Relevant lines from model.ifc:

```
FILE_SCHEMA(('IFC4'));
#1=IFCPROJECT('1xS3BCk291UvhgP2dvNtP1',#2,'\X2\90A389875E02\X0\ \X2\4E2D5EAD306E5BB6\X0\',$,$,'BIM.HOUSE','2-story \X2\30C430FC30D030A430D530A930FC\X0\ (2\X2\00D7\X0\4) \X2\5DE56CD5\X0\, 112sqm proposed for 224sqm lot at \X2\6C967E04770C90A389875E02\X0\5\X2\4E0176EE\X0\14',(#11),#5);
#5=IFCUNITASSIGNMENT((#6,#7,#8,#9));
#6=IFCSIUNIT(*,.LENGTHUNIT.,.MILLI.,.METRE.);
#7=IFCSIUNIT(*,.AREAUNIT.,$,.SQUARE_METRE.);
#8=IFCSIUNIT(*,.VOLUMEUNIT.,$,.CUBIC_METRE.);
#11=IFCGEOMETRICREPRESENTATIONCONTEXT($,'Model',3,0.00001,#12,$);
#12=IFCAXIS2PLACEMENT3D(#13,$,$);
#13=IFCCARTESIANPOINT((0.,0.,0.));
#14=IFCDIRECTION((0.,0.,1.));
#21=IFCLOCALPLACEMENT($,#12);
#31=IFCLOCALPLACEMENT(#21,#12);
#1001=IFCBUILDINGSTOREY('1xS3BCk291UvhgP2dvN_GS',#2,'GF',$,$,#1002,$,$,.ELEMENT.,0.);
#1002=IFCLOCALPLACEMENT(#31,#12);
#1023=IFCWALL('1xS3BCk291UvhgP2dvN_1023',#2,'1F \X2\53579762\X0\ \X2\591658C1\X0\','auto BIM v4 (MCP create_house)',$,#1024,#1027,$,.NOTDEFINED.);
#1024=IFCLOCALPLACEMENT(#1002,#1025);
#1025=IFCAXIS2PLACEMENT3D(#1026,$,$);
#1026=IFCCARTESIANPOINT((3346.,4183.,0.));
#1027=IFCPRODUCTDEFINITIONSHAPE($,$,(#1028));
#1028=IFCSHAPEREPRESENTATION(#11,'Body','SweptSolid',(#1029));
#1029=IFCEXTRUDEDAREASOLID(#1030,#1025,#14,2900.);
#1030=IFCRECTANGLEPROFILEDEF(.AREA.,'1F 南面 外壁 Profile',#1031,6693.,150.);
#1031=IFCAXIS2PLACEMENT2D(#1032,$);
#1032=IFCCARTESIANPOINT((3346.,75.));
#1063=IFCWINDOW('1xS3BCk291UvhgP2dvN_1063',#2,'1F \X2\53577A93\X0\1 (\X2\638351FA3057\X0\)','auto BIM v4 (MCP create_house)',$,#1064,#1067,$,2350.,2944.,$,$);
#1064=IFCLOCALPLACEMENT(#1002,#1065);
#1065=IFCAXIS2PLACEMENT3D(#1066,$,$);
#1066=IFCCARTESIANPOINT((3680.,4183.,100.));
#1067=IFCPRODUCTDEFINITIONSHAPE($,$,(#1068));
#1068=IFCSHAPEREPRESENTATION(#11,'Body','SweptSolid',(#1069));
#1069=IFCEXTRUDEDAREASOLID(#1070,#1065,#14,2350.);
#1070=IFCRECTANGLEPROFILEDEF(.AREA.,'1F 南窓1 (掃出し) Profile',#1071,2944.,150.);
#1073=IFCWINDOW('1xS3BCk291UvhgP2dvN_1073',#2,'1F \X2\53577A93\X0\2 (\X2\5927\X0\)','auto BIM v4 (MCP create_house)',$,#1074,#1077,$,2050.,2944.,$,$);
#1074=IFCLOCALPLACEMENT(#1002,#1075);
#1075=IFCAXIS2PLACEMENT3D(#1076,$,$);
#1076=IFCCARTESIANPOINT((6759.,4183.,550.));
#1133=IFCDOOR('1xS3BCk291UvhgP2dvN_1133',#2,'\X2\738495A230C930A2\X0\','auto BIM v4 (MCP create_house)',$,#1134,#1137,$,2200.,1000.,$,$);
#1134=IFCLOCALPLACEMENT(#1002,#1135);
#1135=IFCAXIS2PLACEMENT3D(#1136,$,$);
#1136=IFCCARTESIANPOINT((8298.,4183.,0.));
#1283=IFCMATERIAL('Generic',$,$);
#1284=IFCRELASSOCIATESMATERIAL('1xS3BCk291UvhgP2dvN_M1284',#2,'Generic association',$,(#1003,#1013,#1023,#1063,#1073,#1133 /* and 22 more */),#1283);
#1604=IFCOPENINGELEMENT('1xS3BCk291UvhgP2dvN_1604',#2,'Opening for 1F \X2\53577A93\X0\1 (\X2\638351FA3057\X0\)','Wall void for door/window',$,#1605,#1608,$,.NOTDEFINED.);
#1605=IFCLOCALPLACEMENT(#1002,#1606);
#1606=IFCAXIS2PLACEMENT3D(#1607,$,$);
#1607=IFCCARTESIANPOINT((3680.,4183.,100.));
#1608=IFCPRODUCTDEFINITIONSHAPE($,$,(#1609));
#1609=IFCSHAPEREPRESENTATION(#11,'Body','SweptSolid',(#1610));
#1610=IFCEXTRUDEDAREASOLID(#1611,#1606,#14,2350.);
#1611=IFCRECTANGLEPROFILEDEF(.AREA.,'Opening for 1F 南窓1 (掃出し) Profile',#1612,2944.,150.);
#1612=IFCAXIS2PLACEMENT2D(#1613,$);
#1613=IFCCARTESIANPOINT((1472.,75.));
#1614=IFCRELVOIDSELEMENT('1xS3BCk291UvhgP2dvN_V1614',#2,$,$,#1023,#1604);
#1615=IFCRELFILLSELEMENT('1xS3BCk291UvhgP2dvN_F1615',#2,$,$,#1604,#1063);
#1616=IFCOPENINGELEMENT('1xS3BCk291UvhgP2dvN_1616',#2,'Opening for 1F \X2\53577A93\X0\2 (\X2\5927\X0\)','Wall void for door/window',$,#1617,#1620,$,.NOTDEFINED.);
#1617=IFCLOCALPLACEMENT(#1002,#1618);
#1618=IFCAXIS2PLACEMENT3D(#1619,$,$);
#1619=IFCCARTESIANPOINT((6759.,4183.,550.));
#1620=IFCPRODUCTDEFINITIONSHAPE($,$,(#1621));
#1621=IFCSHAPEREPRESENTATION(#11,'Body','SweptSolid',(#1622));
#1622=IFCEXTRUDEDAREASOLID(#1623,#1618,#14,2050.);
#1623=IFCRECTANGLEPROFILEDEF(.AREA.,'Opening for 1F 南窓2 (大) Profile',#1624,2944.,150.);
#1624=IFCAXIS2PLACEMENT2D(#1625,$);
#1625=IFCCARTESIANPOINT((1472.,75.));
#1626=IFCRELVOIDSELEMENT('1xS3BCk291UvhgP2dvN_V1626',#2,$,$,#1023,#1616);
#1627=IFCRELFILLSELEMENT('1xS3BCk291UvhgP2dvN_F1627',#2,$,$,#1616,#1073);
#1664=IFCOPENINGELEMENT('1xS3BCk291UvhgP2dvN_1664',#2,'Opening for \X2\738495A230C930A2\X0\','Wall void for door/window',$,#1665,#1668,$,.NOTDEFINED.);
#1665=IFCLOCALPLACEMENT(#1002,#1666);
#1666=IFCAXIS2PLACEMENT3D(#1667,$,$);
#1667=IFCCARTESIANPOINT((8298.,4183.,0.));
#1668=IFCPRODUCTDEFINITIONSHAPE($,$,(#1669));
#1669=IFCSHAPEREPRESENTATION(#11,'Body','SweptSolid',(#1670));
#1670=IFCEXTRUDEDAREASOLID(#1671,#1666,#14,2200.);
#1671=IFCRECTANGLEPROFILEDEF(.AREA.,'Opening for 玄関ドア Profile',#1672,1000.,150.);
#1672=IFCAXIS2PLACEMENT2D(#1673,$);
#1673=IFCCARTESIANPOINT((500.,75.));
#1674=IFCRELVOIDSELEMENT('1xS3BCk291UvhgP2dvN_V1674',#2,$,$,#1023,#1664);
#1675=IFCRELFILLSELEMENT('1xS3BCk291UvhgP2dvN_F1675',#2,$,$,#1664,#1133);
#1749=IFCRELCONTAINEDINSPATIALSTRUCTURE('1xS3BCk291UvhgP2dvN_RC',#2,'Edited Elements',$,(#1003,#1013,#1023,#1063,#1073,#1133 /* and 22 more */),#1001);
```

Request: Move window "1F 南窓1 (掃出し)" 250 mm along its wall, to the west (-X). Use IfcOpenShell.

```python
import ifcopenshell
import ifcopenshell.api.geometry
import ifcopenshell.util.placement

model = ifcopenshell.open("model.ifc")

window = model.by_guid("1xS3BCk291UvhgP2dvN_1063")
opening = window.FillsVoids[0].RelatingOpeningElement
wall = opening.VoidsElements[0].RelatingBuildingElement

wall_matrix = ifcopenshell.util.placement.get_local_placement(wall.ObjectPlacement)
shift = wall_matrix[:3, 0] * -250.0
before = ifcopenshell.util.placement.get_local_placement(window.ObjectPlacement)[:3, 3].copy()

# The window is not placed relative to its opening, so move both.
for product in (opening, window):
    matrix = ifcopenshell.util.placement.get_local_placement(product.ObjectPlacement)
    matrix[:3, 3] += shift
    ifcopenshell.api.geometry.edit_object_placement(model, product=product, matrix=matrix, is_si=False)

after = ifcopenshell.util.placement.get_local_placement(window.ObjectPlacement)[:3, 3]
print("window moved by", (after - before).round(3) + 0.0)

model.write("model_rev.ifc")
```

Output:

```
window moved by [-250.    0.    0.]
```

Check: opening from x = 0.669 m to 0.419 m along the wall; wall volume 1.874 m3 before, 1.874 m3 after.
